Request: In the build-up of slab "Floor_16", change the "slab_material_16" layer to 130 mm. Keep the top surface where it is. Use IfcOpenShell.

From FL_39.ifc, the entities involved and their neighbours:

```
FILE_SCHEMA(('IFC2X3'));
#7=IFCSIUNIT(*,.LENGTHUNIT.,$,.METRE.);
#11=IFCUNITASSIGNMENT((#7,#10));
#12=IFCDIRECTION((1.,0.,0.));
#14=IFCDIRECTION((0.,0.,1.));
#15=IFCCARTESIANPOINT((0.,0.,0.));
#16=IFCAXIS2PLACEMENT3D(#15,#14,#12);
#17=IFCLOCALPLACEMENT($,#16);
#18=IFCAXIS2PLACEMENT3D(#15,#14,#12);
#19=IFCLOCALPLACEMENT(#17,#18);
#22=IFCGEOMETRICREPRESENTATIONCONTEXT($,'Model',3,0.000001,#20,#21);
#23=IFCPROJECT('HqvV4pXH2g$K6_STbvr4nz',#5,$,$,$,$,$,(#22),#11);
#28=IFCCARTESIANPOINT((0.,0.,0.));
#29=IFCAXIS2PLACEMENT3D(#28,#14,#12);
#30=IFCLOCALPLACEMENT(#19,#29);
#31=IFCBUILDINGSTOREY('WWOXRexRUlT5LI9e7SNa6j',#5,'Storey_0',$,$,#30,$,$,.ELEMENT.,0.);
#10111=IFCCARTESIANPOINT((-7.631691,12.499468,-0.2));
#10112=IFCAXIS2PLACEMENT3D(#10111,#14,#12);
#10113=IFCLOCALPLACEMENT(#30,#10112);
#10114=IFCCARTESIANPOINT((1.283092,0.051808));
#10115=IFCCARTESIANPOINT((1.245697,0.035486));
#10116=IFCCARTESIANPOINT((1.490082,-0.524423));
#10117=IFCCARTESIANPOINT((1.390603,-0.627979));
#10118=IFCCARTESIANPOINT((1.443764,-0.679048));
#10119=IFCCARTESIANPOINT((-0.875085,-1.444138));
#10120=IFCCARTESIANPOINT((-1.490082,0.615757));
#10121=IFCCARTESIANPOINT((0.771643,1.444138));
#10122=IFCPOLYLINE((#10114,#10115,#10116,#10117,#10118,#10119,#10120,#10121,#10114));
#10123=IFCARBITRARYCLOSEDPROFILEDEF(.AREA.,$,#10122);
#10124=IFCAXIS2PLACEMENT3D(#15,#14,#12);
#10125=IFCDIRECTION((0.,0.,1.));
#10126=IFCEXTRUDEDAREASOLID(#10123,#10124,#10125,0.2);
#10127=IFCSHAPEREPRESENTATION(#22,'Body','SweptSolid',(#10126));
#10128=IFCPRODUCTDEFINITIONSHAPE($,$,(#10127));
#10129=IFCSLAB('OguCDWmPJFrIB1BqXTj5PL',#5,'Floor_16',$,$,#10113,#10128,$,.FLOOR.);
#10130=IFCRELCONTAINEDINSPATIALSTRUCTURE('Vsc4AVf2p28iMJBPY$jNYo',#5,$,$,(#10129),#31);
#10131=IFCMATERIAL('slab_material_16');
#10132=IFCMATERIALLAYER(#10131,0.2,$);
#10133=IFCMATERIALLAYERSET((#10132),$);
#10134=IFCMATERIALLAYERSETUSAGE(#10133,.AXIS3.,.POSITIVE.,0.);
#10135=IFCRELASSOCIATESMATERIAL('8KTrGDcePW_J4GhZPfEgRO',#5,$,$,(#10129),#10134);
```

```python
import ifcopenshell
import ifcopenshell.util.element
import ifcopenshell.util.unit

model = ifcopenshell.open("FL_39.ifc")
unit_scale = ifcopenshell.util.unit.calculate_unit_scale(model)

layer_set = model.by_id(10133)
layer = next(l for l in layer_set.MaterialLayers if l.Material and l.Material.Name == "slab_material_16")
change = 0.13 / unit_scale - layer.LayerThickness
layer.LayerThickness += change

# Geometry does not follow the layer set by itself.
slabs = [e for e in ifcopenshell.util.element.get_elements_by_material(model, layer_set) if e.is_a("IfcSlab")]
for slab in sorted(slabs, key=lambda e: e.id()):
    body = next(r for r in slab.Representation.Representations if r.RepresentationIdentifier == "Body")
    solid = body.Items[0]
    old_depth = solid.Depth
    solid.Depth += change
    # Extruded upwards: lower the start of the extrusion so the top stays.
    x, y, z = solid.Position.Location.Coordinates
    solid.Position.Location = model.createIfcCartesianPoint((x, y, z - change))
    print(slab.id(), f"{old_depth:g} -> {solid.Depth:g}")

# The layers are counted up from the underside, which has moved.
for usage in {ifcopenshell.util.element.get_material(slab) for slab in slabs}:
    usage.OffsetFromReferenceLine -= change

model.write("FL_39_rev.ifc")
```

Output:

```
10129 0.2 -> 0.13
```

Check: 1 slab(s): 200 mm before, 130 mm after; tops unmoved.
